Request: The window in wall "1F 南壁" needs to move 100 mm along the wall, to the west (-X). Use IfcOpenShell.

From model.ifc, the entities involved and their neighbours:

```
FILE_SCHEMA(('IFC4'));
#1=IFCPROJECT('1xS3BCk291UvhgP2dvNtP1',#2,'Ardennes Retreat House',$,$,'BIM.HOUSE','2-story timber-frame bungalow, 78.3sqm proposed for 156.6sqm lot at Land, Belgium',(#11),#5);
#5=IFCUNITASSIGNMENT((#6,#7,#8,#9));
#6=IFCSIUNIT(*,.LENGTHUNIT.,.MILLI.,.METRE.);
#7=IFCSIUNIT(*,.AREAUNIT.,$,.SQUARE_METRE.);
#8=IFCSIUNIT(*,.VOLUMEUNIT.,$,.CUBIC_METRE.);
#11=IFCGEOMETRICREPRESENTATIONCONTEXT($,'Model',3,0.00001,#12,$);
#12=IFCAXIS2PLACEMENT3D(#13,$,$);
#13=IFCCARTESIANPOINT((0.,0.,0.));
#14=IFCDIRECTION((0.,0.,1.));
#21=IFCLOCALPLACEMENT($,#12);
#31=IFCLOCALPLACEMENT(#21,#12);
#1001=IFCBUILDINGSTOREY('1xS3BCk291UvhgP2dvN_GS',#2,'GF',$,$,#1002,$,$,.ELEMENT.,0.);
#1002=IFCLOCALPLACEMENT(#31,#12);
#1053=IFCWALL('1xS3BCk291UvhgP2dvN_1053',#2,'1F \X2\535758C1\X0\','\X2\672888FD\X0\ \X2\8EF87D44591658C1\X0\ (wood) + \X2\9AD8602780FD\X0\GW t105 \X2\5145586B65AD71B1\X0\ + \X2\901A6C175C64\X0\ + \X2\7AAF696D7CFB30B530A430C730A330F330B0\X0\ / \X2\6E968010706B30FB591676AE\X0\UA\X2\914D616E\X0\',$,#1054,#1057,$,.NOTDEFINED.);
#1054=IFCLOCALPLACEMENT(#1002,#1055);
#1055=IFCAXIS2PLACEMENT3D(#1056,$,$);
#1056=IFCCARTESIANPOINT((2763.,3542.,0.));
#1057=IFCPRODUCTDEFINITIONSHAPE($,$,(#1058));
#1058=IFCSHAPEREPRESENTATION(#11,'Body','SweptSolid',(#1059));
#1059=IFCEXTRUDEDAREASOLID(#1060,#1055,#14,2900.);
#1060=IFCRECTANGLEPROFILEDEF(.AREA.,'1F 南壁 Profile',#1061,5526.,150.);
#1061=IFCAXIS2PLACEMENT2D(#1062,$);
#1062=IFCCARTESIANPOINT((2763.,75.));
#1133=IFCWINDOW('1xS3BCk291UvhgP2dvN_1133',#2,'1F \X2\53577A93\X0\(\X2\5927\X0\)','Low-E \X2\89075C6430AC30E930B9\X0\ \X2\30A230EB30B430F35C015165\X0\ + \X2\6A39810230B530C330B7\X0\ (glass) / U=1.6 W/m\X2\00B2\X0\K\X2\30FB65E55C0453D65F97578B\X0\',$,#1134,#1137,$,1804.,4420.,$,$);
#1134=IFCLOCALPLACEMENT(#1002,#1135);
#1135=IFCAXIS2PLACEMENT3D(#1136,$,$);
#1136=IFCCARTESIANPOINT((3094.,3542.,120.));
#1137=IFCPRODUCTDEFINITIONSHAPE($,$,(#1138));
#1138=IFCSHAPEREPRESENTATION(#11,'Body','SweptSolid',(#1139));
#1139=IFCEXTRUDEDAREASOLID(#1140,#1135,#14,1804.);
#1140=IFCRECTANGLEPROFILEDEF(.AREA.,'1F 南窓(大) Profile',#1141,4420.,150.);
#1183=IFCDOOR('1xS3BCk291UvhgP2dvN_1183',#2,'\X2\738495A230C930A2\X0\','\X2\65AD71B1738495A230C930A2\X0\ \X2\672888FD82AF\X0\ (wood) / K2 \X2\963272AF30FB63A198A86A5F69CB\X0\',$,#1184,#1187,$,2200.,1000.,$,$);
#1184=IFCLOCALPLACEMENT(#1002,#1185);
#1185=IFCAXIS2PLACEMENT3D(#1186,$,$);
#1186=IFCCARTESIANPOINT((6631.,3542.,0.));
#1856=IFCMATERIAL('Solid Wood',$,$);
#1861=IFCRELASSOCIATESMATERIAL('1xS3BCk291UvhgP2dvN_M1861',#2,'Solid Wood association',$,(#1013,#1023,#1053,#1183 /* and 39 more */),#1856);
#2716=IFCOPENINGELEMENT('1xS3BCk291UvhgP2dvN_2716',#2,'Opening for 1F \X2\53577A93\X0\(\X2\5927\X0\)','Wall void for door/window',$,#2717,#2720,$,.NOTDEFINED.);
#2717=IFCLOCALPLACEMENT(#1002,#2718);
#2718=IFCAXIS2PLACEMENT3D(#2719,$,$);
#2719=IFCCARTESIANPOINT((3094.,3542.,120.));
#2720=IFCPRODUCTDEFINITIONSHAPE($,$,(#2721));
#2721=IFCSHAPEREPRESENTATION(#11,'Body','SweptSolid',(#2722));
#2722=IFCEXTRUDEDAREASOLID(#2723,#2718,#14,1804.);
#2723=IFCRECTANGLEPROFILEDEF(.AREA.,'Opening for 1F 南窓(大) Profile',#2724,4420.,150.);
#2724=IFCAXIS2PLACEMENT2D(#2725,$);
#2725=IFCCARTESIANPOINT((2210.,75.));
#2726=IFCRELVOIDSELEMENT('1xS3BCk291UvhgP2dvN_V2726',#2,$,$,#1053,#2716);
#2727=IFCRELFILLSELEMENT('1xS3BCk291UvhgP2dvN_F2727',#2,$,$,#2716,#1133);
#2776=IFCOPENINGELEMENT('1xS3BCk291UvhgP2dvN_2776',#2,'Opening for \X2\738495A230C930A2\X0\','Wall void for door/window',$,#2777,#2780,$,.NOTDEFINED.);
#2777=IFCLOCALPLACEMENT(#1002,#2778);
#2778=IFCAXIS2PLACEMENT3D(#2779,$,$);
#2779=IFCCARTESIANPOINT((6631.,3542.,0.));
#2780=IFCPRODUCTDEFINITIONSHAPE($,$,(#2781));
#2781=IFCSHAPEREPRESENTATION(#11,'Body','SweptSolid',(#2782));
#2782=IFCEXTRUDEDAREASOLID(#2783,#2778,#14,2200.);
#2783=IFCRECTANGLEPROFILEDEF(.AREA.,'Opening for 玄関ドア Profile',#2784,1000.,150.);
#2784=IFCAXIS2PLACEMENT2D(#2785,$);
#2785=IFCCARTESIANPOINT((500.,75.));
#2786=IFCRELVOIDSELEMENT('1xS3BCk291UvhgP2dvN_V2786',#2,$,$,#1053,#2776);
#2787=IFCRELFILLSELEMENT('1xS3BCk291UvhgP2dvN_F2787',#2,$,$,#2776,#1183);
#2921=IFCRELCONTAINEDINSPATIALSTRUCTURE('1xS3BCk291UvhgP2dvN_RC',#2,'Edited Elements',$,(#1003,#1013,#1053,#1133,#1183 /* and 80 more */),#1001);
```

```python
import ifcopenshell
import ifcopenshell.api.geometry
import ifcopenshell.util.placement

model = ifcopenshell.open("model.ifc")

window = model.by_guid("1xS3BCk291UvhgP2dvN_1133")
opening = window.FillsVoids[0].RelatingOpeningElement
wall = opening.VoidsElements[0].RelatingBuildingElement

wall_matrix = ifcopenshell.util.placement.get_local_placement(wall.ObjectPlacement)
shift = wall_matrix[:3, 0] * -100.0
before = ifcopenshell.util.placement.get_local_placement(window.ObjectPlacement)[:3, 3].copy()

# The window is not placed relative to its opening, so move both.
for product in (opening, window):
    matrix = ifcopenshell.util.placement.get_local_placement(product.ObjectPlacement)
    matrix[:3, 3] += shift
    ifcopenshell.api.geometry.edit_object_placement(model, product=product, matrix=matrix, is_si=False)

after = ifcopenshell.util.placement.get_local_placement(window.ObjectPlacement)[:3, 3]
print("window moved by", (after - before).round(3) + 0.0)

model.write("model_v2.ifc")
```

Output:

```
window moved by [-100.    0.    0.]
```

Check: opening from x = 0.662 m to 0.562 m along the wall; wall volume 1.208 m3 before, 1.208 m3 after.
